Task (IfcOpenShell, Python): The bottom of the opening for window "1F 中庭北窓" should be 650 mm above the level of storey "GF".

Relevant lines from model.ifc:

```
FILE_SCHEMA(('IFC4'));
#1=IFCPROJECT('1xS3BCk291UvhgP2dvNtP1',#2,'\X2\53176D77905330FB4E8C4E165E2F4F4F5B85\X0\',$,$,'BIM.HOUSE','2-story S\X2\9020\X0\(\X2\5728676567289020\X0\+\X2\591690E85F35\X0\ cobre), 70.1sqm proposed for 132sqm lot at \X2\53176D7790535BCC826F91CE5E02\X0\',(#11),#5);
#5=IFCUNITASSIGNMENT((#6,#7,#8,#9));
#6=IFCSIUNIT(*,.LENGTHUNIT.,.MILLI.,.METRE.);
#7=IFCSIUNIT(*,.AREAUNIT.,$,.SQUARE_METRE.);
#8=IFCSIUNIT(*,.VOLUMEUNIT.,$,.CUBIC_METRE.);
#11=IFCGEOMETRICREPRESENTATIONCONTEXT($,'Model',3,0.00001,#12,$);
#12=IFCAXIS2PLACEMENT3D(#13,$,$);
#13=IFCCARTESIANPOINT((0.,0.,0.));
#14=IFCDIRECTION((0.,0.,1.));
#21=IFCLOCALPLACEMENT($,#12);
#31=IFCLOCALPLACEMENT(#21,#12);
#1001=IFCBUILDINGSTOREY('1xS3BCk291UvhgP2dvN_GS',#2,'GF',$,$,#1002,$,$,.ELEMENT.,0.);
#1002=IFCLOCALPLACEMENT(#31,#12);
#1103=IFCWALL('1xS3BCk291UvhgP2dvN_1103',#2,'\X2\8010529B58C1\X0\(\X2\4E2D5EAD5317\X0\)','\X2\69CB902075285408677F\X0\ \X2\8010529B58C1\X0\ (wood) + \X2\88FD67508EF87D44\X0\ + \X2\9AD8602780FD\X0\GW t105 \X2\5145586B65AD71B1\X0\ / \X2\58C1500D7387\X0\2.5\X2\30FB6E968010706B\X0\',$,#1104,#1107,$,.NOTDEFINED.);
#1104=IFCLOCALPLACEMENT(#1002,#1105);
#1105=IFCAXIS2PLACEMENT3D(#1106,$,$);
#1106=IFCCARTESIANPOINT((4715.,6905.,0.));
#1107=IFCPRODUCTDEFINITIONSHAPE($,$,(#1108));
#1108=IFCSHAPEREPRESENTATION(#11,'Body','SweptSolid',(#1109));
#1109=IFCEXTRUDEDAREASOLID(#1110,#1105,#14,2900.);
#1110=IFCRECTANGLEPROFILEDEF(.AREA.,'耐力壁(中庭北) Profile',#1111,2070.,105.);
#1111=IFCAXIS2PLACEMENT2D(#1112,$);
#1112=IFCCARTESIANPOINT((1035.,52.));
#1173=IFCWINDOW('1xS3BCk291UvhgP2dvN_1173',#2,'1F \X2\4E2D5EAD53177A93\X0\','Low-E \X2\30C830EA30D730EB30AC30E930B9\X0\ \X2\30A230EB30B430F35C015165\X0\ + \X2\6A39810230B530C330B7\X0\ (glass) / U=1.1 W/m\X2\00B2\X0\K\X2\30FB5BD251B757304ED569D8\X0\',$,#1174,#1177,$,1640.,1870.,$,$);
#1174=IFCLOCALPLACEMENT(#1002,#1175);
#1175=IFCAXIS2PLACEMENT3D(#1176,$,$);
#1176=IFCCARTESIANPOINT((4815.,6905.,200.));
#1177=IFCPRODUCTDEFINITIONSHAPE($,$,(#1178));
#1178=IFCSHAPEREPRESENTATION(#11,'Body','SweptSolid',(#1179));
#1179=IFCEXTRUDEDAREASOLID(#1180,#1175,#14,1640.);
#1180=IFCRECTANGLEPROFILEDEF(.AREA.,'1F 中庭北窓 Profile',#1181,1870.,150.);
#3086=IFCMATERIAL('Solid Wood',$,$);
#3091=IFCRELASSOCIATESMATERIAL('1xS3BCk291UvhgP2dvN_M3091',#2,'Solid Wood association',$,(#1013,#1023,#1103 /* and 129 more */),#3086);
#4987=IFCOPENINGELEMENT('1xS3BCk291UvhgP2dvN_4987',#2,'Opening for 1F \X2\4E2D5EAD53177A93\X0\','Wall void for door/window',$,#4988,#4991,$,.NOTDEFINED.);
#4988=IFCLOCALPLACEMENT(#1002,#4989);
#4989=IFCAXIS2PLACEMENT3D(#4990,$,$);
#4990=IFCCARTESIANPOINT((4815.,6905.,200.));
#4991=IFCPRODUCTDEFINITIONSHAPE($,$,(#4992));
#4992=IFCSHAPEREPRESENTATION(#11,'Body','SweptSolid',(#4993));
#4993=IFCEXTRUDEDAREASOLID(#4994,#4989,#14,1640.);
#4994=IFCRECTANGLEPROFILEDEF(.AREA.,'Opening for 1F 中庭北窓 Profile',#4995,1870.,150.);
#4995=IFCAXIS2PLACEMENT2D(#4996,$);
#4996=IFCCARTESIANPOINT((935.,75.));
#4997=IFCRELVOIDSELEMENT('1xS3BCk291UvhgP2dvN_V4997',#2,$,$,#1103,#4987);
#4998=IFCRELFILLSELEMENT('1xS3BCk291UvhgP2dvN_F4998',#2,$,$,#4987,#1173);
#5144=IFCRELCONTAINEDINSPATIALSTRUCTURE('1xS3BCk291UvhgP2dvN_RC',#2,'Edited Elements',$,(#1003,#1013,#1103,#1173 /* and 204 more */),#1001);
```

```python
import numpy as np
import ifcopenshell
import ifcopenshell.api.geometry
import ifcopenshell.geom
import ifcopenshell.util.element
import ifcopenshell.util.placement
import ifcopenshell.util.shape
import ifcopenshell.util.unit

model = ifcopenshell.open("model.ifc")
unit_scale = ifcopenshell.util.unit.calculate_unit_scale(model)

window = model.by_guid("1xS3BCk291UvhgP2dvN_1173")
opening = window.FillsVoids[0].RelatingOpeningElement
storey = ifcopenshell.util.element.get_container(window, ifc_class="IfcBuildingStorey")
level = ifcopenshell.util.placement.get_local_placement(storey.ObjectPlacement)[2, 3]

# The opening's origin need not be at the sill, so measure its lowest point.
shape = ifcopenshell.geom.create_shape(ifcopenshell.geom.settings(), opening)
bottom = ifcopenshell.util.shape.get_shape_bottom_elevation(shape, shape.geometry) / unit_scale
dz = level + 650.0 - bottom

shift = np.array([0.0, 0.0, dz])
# The window is not placed relative to its opening, so move both.
for product in (opening, window):
    matrix = ifcopenshell.util.placement.get_local_placement(product.ObjectPlacement)
    matrix[:3, 3] += shift
    ifcopenshell.api.geometry.edit_object_placement(model, product=product, matrix=matrix, is_si=False)

print(f"moved by {dz * unit_scale:+.3f} m")

model.write("model_edited.ifc")
```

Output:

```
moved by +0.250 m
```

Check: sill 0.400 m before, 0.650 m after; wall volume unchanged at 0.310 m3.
